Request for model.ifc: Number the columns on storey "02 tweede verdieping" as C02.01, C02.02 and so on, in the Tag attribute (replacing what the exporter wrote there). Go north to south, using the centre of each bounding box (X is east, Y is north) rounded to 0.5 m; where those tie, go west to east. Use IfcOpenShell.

First a look at what the model holds.

```python
import ifcopenshell
import ifcopenshell.util.element
import ifcopenshell.util.placement

model = ifcopenshell.open("model.ifc")
print(model.schema)
storey = next(s for s in model.by_type("IfcBuildingStorey") if s.Name == "02 tweede verdieping")
columns = [e for e in ifcopenshell.util.element.get_decomposition(storey) if e.is_a("IfcColumn")]
for e in sorted(columns, key=lambda e: e.id()):
    origin = ifcopenshell.util.placement.get_local_placement(e.ObjectPlacement)[:3, 3]
    print(e.id(), e.Tag, e.Name, origin.round(2) + 0.0, sep=" | ")
```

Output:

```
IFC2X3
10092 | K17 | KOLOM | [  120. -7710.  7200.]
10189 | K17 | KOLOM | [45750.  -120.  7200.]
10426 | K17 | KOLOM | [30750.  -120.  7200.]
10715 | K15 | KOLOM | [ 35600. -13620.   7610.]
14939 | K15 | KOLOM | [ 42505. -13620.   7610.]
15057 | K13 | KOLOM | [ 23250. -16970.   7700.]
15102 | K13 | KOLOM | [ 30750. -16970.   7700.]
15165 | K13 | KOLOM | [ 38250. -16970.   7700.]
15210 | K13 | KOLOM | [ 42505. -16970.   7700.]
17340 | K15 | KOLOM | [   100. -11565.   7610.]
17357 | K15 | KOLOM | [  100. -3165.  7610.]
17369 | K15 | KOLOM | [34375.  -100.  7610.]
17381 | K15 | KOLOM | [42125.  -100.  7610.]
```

```python
import ifcopenshell
import ifcopenshell.geom
import ifcopenshell.util.element
import ifcopenshell.util.shape

model = ifcopenshell.open("model.ifc")
settings = ifcopenshell.geom.settings()
settings.set("use-world-coords", True)


def centre(element):
    shape = ifcopenshell.geom.create_shape(settings, element)
    return ifcopenshell.util.shape.get_bbox_centroid(shape.geometry)


storey = next(s for s in model.by_type("IfcBuildingStorey") if s.Name == "02 tweede verdieping")
columns = [e for e in ifcopenshell.util.element.get_decomposition(storey) if e.is_a("IfcColumn")]

# Insertion points can sit at a corner or the storey origin, so sort by the geometry (in metres).
centres = {e: centre(e) for e in columns}
columns.sort(key=lambda e: (-round(centres[e][1] / 0.5), centres[e][0]))

for i, e in enumerate(columns, start=1):
    number = f"C02.{i:02d}"
    e.Tag = number
    print(e.id(), number)

model.write("model-out.ifc")
```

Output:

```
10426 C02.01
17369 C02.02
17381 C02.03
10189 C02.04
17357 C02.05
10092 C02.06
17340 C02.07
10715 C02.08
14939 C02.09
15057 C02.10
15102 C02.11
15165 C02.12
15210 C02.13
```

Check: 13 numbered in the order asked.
